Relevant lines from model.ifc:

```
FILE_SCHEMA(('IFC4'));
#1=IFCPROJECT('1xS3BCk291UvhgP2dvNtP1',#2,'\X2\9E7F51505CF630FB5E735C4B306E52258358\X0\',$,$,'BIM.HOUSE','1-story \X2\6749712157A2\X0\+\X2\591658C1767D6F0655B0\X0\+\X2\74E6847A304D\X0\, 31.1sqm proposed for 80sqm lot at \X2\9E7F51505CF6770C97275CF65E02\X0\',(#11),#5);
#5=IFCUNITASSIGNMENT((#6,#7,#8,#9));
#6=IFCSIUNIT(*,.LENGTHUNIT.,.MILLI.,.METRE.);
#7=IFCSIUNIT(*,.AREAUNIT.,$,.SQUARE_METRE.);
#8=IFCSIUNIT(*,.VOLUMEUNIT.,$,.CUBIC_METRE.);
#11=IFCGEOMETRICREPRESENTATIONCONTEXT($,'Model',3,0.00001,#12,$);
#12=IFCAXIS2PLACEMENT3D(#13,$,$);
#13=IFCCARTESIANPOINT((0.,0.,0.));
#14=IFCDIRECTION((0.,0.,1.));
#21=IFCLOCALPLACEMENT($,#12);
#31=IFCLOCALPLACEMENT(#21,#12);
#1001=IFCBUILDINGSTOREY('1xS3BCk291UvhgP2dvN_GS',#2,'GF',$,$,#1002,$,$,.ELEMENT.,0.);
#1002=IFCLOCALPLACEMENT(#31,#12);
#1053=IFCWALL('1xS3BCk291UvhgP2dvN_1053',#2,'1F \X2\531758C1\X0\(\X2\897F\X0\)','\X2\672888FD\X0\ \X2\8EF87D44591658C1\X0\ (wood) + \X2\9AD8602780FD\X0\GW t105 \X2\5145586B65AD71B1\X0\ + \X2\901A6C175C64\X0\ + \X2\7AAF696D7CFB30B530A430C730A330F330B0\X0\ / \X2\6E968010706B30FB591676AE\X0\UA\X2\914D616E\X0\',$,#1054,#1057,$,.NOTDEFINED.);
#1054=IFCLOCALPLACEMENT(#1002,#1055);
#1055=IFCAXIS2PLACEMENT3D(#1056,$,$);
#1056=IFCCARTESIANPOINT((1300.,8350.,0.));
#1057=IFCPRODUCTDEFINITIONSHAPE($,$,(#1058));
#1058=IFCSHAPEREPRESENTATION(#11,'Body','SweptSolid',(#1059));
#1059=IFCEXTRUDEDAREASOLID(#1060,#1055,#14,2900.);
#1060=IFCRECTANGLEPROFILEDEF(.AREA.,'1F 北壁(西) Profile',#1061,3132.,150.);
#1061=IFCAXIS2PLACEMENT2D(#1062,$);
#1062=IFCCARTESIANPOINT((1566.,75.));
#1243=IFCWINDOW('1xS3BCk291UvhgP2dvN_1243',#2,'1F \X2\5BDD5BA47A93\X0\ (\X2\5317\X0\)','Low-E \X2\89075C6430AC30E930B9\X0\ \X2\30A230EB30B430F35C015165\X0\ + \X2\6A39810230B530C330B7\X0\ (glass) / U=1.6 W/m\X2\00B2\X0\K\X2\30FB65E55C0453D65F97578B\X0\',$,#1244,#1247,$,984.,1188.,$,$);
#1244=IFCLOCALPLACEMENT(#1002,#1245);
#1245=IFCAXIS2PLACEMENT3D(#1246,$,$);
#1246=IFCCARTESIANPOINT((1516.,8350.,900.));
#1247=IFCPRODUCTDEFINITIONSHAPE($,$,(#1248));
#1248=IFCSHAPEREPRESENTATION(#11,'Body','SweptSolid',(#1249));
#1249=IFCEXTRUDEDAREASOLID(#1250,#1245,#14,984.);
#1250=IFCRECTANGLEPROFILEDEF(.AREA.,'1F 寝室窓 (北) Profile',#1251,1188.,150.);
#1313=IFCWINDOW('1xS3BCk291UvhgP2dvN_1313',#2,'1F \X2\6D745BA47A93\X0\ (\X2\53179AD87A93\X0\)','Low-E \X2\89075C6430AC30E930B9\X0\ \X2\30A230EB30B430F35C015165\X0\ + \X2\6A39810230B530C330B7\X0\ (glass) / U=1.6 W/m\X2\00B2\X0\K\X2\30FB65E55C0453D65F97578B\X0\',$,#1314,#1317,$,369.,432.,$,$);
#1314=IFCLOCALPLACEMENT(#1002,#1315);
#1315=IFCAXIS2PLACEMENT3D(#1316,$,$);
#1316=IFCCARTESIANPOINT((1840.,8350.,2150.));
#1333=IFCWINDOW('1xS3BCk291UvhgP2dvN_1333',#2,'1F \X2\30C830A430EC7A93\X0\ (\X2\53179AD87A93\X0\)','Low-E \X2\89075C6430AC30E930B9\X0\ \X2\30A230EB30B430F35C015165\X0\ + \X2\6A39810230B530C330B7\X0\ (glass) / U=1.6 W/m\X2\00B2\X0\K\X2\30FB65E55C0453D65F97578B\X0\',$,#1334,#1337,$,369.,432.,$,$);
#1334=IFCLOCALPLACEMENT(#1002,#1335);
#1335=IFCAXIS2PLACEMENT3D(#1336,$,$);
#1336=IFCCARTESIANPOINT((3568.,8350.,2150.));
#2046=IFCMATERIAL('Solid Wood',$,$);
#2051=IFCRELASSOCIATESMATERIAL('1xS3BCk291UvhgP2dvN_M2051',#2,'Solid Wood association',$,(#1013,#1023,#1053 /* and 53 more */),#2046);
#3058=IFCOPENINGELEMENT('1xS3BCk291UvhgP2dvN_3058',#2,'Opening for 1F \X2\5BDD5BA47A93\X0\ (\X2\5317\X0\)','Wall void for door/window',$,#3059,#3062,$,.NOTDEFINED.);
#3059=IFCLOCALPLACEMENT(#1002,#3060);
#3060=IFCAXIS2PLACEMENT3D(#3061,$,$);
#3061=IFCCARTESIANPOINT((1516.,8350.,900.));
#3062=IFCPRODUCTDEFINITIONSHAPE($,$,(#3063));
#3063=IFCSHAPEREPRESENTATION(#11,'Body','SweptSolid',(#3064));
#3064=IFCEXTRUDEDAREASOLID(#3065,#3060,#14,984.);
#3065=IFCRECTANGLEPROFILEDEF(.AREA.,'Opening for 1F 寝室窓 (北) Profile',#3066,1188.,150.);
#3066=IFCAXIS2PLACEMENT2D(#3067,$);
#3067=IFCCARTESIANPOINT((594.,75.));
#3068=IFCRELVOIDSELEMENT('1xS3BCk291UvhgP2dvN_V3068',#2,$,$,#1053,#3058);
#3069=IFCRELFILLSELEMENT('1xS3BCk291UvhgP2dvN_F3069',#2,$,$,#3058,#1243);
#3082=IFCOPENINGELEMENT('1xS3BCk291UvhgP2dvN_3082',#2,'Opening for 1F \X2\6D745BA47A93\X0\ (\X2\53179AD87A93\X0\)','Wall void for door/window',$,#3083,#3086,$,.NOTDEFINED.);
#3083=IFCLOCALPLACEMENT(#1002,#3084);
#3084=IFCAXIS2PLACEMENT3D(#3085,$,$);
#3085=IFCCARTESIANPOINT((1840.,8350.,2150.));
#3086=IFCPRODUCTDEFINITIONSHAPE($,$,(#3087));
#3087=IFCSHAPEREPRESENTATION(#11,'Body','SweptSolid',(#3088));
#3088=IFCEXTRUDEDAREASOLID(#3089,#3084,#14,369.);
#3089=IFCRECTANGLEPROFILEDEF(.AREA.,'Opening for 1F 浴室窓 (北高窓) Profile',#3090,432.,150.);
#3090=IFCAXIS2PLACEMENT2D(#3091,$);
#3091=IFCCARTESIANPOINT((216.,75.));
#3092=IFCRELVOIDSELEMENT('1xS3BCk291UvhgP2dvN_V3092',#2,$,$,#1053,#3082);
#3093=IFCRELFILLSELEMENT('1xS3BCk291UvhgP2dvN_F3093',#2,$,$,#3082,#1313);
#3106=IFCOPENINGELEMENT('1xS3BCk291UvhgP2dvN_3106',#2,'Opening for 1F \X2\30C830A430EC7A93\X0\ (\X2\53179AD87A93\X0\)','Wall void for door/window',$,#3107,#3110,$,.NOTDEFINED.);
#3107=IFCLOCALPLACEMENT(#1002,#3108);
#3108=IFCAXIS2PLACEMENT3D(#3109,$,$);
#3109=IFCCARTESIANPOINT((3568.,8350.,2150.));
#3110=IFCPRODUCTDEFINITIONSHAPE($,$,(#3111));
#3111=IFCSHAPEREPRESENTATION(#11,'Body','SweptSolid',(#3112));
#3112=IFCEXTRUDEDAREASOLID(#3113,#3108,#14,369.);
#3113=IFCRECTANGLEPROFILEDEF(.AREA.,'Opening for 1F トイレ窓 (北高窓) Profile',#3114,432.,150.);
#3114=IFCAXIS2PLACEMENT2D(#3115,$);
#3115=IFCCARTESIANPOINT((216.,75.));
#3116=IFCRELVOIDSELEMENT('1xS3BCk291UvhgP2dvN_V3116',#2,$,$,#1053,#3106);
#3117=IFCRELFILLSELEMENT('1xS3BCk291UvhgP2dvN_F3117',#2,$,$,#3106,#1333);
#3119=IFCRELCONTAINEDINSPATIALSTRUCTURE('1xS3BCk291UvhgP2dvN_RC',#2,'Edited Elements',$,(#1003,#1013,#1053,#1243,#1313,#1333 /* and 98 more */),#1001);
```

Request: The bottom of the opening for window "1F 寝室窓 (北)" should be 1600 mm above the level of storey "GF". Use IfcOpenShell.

```python
import numpy as np
import ifcopenshell
import ifcopenshell.api.geometry
import ifcopenshell.geom
import ifcopenshell.util.element
import ifcopenshell.util.placement
import ifcopenshell.util.shape
import ifcopenshell.util.unit

model = ifcopenshell.open("model.ifc")
unit_scale = ifcopenshell.util.unit.calculate_unit_scale(model)

window = model.by_guid("1xS3BCk291UvhgP2dvN_1243")
opening = window.FillsVoids[0].RelatingOpeningElement
storey = ifcopenshell.util.element.get_container(window, ifc_class="IfcBuildingStorey")
level = ifcopenshell.util.placement.get_local_placement(storey.ObjectPlacement)[2, 3]

# The opening's origin need not be at the sill, so measure its lowest point.
shape = ifcopenshell.geom.create_shape(ifcopenshell.geom.settings(), opening)
bottom = ifcopenshell.util.shape.get_shape_bottom_elevation(shape, shape.geometry) / unit_scale
dz = level + 1.6 / unit_scale - bottom

shift = np.array([0.0, 0.0, dz])
# The window is not placed relative to its opening, so move both.
for product in (opening, window):
    matrix = ifcopenshell.util.placement.get_local_placement(product.ObjectPlacement)
    matrix[:3, 3] += shift
    ifcopenshell.api.geometry.edit_object_placement(model, product=product, matrix=matrix, is_si=False)

print(f"moved by {dz * unit_scale:+.3f} m")

model.write("model_edited.ifc")
```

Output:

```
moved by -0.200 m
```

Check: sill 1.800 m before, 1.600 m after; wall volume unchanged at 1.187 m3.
